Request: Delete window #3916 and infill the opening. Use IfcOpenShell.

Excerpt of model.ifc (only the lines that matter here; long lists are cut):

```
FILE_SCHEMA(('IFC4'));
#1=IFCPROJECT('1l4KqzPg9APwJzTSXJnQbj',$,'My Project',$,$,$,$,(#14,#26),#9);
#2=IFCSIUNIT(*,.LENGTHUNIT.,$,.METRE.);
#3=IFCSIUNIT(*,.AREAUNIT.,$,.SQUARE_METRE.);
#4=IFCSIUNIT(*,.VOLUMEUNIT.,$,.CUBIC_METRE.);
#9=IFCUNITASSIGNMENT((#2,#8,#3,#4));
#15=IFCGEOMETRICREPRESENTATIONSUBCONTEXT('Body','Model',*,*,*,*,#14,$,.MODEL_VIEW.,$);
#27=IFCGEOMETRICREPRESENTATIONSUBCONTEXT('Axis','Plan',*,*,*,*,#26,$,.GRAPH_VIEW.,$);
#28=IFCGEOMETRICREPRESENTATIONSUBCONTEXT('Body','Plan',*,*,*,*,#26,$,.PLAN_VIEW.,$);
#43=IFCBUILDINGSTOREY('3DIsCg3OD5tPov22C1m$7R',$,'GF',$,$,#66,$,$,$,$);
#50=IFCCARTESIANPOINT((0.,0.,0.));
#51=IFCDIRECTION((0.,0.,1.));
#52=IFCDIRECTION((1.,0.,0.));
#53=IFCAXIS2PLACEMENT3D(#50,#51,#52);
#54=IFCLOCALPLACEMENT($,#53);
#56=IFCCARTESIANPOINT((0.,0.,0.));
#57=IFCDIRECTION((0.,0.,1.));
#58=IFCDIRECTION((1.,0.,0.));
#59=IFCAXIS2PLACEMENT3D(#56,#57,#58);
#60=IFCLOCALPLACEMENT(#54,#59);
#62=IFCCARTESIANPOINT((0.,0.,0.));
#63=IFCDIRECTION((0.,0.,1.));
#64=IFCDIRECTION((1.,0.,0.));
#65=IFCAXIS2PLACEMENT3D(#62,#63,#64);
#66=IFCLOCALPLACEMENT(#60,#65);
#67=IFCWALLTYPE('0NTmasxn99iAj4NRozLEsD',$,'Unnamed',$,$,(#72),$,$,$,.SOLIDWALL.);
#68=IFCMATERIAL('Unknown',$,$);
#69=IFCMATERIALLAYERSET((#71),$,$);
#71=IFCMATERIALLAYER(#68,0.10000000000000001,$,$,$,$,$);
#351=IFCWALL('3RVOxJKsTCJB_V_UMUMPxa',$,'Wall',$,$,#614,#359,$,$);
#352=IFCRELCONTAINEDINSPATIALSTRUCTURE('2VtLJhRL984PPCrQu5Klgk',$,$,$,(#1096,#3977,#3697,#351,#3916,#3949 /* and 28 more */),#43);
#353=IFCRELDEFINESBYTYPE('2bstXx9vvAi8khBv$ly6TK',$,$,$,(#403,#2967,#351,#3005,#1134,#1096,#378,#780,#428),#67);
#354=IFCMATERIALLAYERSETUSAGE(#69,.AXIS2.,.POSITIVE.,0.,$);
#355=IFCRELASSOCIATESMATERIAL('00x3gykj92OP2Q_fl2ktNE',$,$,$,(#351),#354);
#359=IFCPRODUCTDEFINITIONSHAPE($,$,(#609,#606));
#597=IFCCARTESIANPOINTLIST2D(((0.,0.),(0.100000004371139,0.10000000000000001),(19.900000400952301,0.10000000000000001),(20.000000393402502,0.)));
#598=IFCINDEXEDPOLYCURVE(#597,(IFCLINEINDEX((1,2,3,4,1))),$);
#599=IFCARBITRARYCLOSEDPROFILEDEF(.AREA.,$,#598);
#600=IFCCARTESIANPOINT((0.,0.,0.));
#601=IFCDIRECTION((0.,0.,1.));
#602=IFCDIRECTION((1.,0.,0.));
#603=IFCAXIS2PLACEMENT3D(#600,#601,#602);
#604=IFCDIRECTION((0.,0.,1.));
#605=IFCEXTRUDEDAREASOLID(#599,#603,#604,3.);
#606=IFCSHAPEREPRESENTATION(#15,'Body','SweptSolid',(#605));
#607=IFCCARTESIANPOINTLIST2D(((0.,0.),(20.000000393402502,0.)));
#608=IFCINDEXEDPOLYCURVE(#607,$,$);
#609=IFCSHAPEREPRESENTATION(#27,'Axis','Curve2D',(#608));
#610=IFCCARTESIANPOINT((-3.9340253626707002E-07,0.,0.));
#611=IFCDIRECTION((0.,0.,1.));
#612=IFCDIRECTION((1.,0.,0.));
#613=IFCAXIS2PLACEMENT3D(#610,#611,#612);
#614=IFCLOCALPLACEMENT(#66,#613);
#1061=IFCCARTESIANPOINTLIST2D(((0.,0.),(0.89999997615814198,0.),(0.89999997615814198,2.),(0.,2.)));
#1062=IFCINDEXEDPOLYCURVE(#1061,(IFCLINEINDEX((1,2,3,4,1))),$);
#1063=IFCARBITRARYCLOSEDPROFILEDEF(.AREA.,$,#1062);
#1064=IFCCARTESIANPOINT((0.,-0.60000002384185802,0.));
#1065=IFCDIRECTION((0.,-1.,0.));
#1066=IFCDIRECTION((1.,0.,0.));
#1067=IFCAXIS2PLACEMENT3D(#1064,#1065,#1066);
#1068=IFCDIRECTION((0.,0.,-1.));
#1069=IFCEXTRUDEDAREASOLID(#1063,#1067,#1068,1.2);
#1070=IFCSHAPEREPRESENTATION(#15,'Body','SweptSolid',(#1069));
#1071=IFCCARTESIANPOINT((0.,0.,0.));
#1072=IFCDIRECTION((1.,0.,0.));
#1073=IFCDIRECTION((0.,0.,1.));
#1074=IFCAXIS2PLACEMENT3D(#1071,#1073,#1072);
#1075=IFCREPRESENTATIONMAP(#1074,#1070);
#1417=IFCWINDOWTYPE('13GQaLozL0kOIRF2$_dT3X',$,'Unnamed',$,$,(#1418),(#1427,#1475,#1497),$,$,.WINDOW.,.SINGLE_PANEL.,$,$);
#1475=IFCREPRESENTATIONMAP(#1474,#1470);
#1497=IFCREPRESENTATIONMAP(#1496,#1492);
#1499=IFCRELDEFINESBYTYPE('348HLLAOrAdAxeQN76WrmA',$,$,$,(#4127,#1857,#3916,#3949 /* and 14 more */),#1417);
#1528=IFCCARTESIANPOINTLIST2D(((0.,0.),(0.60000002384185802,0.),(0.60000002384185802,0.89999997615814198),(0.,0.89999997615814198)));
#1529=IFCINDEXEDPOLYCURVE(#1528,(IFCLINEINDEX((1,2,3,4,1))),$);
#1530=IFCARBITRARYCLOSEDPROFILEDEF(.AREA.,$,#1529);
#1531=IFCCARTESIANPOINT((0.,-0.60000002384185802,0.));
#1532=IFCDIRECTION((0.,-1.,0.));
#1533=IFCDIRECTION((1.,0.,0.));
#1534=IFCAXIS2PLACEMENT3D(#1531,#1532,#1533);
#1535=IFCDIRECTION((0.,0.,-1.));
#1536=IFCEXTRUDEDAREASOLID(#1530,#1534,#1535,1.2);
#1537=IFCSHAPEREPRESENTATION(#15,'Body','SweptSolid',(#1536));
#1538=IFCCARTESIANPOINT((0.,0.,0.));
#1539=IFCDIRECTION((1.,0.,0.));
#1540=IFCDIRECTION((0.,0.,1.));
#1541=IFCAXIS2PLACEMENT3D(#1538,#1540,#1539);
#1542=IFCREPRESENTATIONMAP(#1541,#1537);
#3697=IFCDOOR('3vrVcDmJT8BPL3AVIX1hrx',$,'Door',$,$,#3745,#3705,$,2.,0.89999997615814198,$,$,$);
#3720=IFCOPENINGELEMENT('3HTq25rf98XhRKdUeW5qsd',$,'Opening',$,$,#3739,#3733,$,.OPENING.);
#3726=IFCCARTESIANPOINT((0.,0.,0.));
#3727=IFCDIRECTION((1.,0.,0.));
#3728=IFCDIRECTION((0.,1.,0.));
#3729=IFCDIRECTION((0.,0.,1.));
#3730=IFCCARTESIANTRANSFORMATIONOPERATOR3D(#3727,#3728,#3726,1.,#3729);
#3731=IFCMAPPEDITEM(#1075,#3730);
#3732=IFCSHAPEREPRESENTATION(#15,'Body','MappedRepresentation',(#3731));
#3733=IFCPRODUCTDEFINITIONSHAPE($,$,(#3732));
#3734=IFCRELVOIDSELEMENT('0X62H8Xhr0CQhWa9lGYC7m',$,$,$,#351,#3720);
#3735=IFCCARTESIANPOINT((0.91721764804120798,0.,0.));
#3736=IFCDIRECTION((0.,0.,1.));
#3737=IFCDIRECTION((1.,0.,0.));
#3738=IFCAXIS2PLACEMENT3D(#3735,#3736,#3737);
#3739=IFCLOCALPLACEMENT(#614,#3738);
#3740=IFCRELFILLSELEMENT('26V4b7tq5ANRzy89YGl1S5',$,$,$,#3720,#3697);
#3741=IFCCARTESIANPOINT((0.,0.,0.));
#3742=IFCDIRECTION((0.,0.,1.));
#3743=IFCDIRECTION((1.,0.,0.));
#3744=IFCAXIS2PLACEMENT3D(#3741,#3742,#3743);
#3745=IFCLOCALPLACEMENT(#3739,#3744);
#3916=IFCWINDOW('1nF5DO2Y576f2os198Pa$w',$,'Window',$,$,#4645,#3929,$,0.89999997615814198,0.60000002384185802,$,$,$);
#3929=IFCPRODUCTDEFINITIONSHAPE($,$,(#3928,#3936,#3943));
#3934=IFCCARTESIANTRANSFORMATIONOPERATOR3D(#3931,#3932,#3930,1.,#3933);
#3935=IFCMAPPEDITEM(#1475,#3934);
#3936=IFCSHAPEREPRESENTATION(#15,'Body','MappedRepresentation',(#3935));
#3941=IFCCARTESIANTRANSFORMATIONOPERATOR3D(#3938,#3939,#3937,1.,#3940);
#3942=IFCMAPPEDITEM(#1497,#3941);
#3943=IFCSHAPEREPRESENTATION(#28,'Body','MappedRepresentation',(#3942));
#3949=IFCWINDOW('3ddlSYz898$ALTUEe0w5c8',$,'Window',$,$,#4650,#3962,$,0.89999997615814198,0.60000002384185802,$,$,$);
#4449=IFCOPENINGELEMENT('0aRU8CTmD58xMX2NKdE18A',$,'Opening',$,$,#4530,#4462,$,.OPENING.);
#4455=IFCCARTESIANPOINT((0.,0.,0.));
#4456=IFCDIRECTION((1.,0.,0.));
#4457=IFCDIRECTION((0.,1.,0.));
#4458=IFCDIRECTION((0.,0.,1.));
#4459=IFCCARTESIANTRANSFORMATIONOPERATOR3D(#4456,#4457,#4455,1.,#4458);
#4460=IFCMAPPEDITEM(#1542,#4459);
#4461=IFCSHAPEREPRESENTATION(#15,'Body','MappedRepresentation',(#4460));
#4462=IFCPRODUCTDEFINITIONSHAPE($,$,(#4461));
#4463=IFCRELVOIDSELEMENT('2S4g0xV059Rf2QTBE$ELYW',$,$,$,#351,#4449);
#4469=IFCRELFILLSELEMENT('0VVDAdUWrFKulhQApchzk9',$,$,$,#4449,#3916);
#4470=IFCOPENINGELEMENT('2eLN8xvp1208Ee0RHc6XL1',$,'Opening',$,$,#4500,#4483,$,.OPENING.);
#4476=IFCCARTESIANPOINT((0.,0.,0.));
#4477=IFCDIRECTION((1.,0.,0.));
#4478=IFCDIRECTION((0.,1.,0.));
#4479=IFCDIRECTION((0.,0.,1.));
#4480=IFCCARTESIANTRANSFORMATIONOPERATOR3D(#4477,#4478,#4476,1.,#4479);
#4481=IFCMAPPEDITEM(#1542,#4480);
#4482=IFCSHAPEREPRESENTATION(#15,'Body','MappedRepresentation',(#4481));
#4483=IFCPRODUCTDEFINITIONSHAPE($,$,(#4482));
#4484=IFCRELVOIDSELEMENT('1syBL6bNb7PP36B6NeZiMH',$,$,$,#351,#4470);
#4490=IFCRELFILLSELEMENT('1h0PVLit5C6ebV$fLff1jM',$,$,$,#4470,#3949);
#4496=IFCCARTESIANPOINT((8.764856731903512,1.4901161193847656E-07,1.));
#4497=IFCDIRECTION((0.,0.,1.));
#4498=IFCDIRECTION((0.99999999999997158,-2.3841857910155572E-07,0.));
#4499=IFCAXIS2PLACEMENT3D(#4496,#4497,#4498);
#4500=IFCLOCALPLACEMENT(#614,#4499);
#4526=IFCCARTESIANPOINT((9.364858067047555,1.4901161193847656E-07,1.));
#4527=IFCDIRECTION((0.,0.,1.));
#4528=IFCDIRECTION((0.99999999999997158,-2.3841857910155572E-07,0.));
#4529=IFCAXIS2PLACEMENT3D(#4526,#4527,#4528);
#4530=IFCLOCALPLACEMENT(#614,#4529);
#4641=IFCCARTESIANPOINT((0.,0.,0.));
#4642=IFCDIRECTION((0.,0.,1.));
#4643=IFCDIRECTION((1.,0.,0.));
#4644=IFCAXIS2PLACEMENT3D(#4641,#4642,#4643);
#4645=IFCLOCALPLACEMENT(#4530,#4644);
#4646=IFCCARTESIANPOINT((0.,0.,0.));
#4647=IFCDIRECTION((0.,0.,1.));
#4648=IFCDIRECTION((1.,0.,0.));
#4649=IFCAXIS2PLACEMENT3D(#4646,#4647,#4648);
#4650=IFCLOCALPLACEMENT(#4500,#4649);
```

```python
import ifcopenshell
import ifcopenshell.api.feature
import ifcopenshell.api.root
import ifcopenshell.geom
import ifcopenshell.util.shape

model = ifcopenshell.open("model.ifc")
settings = ifcopenshell.geom.settings()


def volume(element):
    """Net volume in cubic metres, openings subtracted."""
    shape = ifcopenshell.geom.create_shape(settings, element)
    return ifcopenshell.util.shape.get_volume(shape.geometry)


window = model.by_id(3916)
opening = window.FillsVoids[0].RelatingOpeningElement
wall = opening.VoidsElements[0].RelatingBuildingElement
before = volume(wall)

ifcopenshell.api.root.remove_product(model, product=window)
ifcopenshell.api.feature.remove_feature(model, feature=opening)

after = volume(wall)

print(f"wall volume {before:.3f} -> {after:.3f} m3")

model.write("model-out.ifc")
```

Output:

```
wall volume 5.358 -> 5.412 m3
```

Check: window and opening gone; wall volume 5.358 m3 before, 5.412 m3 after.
